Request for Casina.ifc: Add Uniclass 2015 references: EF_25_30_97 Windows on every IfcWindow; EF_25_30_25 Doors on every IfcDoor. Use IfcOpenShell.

First a look at what the model holds.

```python
import ifcopenshell

model = ifcopenshell.open("Casina.ifc")
print(model.schema)
print("classifications:", [c.Name for c in model.by_type("IfcClassification")])
for ifc_class in ("IfcDoor", "IfcRoof", "IfcStair", "IfcWall", "IfcWindow"):
    print(ifc_class, len(model.by_type(ifc_class)))
```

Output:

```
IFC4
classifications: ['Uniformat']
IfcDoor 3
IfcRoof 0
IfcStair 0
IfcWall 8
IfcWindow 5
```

```python
import ifcopenshell
import ifcopenshell.api.classification

model = ifcopenshell.open("Casina.ifc")

system = ifcopenshell.api.classification.add_classification(model, classification="Uniclass 2015")

codes = {
    "IfcWindow": ("EF_25_30_97", "Windows"),
    "IfcDoor": ("EF_25_30_25", "Doors"),
}
for ifc_class, (code, name) in codes.items():
    products = model.by_type(ifc_class)
    ifcopenshell.api.classification.add_reference(
        model, products=products, classification=system, identification=code, name=name
    )
    print(code, len(products))

model.write("Casina_updated.ifc")
```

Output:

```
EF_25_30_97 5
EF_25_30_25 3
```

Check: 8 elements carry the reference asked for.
